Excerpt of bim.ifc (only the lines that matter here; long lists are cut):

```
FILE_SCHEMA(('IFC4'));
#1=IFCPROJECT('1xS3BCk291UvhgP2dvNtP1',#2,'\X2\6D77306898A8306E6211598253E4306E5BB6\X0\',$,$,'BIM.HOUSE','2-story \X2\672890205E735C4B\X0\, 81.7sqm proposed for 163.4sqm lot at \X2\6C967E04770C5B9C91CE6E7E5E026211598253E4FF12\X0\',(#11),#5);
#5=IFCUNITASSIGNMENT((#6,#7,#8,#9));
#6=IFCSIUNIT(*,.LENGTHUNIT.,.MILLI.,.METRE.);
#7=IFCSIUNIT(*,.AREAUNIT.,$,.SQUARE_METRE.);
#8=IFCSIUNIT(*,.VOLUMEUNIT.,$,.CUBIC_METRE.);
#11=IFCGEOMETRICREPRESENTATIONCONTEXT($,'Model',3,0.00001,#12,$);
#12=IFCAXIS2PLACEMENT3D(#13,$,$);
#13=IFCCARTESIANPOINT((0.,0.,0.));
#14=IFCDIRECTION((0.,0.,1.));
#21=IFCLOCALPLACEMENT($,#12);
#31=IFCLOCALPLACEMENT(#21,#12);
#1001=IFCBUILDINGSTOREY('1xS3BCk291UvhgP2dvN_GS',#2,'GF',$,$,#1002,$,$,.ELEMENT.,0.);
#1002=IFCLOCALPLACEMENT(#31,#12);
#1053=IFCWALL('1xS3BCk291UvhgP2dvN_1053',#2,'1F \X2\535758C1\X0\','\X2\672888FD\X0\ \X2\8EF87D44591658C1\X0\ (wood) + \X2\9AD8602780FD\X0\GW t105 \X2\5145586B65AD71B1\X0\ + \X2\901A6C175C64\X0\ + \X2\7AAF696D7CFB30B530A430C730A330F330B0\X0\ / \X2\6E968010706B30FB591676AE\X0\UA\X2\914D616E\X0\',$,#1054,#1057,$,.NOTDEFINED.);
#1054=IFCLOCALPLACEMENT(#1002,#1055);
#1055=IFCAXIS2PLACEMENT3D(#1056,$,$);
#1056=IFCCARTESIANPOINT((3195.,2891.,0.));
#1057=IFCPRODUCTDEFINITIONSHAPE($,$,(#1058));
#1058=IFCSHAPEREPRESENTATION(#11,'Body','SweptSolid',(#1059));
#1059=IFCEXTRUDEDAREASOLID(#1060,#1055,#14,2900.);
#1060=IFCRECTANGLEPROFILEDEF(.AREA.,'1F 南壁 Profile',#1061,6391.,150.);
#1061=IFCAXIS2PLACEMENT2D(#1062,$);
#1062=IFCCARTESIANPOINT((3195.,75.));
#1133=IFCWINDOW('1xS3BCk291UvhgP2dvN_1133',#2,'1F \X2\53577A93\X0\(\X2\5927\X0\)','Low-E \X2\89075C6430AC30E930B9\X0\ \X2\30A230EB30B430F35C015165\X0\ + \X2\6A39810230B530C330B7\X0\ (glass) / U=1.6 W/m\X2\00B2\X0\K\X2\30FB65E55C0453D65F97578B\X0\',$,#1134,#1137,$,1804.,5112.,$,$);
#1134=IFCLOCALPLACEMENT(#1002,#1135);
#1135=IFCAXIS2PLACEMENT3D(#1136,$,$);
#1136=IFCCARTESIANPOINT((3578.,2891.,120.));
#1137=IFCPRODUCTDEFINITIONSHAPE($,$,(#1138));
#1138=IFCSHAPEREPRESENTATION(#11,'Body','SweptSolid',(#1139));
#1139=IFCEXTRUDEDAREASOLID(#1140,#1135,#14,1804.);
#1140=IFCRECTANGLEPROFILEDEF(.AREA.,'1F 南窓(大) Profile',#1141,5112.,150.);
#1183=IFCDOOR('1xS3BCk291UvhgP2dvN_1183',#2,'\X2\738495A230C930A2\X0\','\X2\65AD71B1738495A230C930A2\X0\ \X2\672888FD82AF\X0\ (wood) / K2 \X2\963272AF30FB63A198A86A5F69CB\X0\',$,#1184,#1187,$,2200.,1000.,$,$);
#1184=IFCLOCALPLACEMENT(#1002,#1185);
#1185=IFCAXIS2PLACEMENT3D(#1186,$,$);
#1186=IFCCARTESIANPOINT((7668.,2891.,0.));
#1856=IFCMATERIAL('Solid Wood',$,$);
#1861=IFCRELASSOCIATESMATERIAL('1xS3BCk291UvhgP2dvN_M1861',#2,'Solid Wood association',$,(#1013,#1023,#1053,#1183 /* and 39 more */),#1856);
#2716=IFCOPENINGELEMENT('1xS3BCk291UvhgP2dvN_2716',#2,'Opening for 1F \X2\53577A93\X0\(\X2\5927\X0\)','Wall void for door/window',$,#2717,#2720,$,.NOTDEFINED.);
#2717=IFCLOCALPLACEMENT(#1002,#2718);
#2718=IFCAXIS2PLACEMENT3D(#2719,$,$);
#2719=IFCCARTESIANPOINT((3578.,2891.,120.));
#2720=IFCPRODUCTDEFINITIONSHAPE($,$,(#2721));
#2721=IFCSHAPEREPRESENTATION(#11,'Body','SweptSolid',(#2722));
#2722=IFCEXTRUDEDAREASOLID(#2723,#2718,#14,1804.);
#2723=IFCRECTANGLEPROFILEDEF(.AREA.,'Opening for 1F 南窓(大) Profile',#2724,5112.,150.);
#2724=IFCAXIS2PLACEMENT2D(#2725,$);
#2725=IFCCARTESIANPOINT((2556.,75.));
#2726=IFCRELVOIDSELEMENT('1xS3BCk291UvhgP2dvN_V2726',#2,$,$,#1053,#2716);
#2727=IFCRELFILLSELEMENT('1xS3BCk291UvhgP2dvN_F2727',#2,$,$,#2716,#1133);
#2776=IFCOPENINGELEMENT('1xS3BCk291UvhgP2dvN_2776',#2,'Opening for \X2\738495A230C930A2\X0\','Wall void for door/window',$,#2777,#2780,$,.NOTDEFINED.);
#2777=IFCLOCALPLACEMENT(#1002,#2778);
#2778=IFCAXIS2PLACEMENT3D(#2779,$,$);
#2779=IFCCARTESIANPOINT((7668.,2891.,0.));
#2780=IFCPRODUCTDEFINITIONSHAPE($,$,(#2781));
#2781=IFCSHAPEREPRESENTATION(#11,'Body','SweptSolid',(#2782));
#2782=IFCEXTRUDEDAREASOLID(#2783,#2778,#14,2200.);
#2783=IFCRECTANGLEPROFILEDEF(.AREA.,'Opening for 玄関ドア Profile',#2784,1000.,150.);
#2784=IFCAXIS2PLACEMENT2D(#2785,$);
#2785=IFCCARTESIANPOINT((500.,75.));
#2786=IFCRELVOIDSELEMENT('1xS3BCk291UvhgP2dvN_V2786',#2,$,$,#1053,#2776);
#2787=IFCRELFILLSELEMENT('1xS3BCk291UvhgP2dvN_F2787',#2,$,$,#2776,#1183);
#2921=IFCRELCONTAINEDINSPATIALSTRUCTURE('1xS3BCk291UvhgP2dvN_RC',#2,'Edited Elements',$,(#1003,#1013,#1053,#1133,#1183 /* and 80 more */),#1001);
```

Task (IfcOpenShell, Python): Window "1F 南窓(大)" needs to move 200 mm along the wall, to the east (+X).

```python
import ifcopenshell
import ifcopenshell.api.geometry
import ifcopenshell.util.placement

model = ifcopenshell.open("bim.ifc")

window = model.by_id(1133)
opening = window.FillsVoids[0].RelatingOpeningElement
wall = opening.VoidsElements[0].RelatingBuildingElement

wall_matrix = ifcopenshell.util.placement.get_local_placement(wall.ObjectPlacement)
shift = wall_matrix[:3, 0] * 200.0
before = ifcopenshell.util.placement.get_local_placement(window.ObjectPlacement)[:3, 3].copy()

# The window is not placed relative to its opening, so move both.
for product in (opening, window):
    matrix = ifcopenshell.util.placement.get_local_placement(product.ObjectPlacement)
    matrix[:3, 3] += shift
    ifcopenshell.api.geometry.edit_object_placement(model, product=product, matrix=matrix, is_si=False)

after = ifcopenshell.util.placement.get_local_placement(window.ObjectPlacement)[:3, 3]
print("window moved by", (after - before).round(3) + 0.0)

model.write("bim_edited.ifc")
```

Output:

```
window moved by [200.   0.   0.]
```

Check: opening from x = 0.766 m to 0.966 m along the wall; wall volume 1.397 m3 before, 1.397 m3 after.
